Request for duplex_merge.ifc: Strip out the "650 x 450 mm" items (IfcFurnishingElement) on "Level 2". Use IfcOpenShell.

First a look at what the model holds.

```python
import ifcopenshell
import ifcopenshell.util.element

model = ifcopenshell.open("duplex_merge.ifc")
print(model.schema)
storey = next(s for s in model.by_type("IfcBuildingStorey") if s.Name == "Level 2")
furniture = [e for e in ifcopenshell.util.element.get_decomposition(storey) if e.is_a("IfcFurnishingElement")]
seen = {}
for e in furniture:
    element_type = ifcopenshell.util.element.get_type(e)
    name = element_type.Name if element_type not in (None, e) else None
    seen[name] = seen.get(name, 0) + 1
for name, count in sorted(seen.items(), key=str):
    print(count, "x", name)
```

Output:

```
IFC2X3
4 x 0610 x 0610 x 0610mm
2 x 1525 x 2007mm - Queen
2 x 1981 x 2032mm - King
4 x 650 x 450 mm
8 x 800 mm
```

```python
import ifcopenshell
import ifcopenshell.api.root
import ifcopenshell.util.element

model = ifcopenshell.open("duplex_merge.ifc")

storey = next(s for s in model.by_type("IfcBuildingStorey") if s.Name == "Level 2")
furniture = [e for e in ifcopenshell.util.element.get_decomposition(storey) if e.is_a("IfcFurnishingElement")]
targets = [e for e in furniture if (t := ifcopenshell.util.element.get_type(e)) not in (None, e) and t.Name == "650 x 450 mm"]

for e in targets:
    ifcopenshell.api.root.remove_product(model, product=e)
print(len(targets), "removed")

model.write("duplex_merge_rev.ifc")
```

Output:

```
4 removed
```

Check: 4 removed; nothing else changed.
